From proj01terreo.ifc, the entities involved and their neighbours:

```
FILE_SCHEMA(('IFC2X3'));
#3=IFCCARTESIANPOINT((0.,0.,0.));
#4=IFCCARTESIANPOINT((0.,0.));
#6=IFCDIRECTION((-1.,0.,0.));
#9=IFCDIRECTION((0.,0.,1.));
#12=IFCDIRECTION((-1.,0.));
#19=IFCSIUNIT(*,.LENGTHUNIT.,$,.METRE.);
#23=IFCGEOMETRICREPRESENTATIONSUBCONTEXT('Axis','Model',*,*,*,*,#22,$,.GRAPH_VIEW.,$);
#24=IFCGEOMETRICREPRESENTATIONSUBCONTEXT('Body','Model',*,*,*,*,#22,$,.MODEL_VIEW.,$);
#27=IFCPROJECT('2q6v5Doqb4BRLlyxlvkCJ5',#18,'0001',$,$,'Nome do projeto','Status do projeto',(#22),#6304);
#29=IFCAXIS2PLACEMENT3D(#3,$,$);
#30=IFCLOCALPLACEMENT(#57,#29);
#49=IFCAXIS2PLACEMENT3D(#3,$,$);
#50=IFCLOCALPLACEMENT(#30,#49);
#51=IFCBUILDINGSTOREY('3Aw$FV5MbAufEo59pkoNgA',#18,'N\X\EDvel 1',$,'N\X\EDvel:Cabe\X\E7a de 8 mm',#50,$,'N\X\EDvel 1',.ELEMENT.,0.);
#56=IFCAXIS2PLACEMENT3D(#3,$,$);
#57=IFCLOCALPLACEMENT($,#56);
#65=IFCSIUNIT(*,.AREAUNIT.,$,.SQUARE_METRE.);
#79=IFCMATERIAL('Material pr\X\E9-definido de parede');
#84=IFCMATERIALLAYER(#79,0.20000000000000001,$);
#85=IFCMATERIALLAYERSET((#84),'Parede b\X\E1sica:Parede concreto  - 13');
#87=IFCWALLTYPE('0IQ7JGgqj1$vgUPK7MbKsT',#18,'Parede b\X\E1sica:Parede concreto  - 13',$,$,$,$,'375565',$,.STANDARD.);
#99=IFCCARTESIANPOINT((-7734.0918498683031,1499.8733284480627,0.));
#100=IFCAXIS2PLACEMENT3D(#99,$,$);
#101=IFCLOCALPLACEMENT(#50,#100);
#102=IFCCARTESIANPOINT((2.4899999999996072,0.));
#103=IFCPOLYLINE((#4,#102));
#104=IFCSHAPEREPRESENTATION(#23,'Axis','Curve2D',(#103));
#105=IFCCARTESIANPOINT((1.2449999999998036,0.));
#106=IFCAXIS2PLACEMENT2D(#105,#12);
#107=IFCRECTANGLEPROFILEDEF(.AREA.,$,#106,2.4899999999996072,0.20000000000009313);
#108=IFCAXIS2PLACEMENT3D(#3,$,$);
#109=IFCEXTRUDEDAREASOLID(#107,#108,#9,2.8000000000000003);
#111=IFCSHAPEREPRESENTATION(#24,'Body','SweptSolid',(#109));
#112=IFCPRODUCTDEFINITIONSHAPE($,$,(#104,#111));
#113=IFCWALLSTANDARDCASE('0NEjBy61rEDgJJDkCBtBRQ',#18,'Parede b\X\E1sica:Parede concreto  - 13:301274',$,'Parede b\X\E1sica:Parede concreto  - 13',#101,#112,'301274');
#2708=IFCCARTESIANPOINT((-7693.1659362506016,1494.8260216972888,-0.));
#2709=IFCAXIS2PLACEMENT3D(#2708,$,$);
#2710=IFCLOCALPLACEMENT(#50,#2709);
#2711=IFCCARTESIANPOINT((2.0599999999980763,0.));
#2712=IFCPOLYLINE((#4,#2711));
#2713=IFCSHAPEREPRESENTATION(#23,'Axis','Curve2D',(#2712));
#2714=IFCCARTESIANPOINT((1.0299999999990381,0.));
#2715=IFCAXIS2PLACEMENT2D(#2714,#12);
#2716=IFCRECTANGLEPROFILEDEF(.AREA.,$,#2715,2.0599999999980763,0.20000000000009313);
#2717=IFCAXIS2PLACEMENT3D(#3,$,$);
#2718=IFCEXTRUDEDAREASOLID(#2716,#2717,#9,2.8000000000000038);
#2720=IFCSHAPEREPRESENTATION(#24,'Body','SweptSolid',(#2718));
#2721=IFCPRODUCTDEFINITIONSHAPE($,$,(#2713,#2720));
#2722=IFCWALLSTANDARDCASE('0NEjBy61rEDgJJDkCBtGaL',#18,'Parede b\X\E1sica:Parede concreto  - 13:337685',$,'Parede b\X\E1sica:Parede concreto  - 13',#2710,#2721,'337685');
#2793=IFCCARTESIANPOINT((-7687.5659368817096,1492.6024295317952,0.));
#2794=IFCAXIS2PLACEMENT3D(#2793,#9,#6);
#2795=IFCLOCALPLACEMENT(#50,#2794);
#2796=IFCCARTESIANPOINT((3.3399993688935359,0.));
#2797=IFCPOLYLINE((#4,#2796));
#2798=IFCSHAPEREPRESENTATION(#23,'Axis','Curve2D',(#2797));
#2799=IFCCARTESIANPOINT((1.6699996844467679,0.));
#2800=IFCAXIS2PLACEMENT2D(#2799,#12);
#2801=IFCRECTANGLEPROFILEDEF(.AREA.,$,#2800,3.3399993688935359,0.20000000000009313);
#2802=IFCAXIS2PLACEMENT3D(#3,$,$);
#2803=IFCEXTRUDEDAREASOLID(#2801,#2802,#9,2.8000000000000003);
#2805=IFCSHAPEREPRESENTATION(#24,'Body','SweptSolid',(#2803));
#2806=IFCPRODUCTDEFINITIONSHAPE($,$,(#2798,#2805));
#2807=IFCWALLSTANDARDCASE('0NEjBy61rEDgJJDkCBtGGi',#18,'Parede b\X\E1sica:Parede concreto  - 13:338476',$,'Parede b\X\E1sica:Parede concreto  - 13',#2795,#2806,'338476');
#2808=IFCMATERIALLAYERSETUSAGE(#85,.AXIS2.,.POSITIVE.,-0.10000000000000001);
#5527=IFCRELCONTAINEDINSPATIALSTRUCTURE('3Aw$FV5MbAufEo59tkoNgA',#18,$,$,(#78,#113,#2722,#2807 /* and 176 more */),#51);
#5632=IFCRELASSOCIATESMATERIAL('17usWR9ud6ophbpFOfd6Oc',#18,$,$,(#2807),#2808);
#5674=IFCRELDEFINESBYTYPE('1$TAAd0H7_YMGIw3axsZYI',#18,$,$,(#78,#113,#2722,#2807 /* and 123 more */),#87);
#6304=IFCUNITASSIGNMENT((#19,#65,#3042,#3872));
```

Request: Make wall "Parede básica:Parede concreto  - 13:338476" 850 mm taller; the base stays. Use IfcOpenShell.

```python
import ifcopenshell
import ifcopenshell.geom
import ifcopenshell.util.representation
import ifcopenshell.util.shape
import ifcopenshell.util.unit

model = ifcopenshell.open("proj01terreo.ifc")
unit_scale = ifcopenshell.util.unit.calculate_unit_scale(model)
settings = ifcopenshell.geom.settings()


def volume(element):
    """Net volume in cubic metres, openings subtracted."""
    shape = ifcopenshell.geom.create_shape(settings, element)
    return ifcopenshell.util.shape.get_volume(shape.geometry)


wall = model.by_guid("0NEjBy61rEDgJJDkCBtGGi")
before = volume(wall)

body = ifcopenshell.util.representation.get_representation(wall, "Model", "Body")
solid = body.Items[0]
old_height = solid.Depth
solid.Depth += 0.85 / unit_scale
after = volume(wall)

print(f"height {old_height:g} -> {solid.Depth:g}, volume {before:.3f} -> {after:.3f} m3")

model.write("proj01terreo_v2.ifc")
```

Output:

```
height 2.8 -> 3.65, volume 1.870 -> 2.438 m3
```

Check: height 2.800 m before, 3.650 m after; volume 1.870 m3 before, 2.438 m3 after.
